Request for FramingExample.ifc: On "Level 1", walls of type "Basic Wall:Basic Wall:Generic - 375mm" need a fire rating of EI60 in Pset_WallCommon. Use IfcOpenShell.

First a look at what the model holds.

```python
import ifcopenshell
import ifcopenshell.util.element

model = ifcopenshell.open("FramingExample.ifc")
print(model.schema)
storey = next(s for s in model.by_type("IfcBuildingStorey") if s.Name == "Level 1")
walls = [e for e in ifcopenshell.util.element.get_decomposition(storey) if e.is_a("IfcWall")]
seen = {}
for e in walls:
    element_type = ifcopenshell.util.element.get_type(e)
    key = (element_type.Name if element_type != e and element_type else None, ifcopenshell.util.element.get_pset(e, "Pset_WallCommon", "FireRating"))
    seen[key] = seen.get(key, 0) + 1
for (name, value), count in sorted(seen.items(), key=str):
    print(count, "x", name, "|", value)
```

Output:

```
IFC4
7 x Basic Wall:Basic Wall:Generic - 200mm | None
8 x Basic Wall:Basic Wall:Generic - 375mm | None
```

```python
import ifcopenshell
import ifcopenshell.api.pset
import ifcopenshell.util.element

model = ifcopenshell.open("FramingExample.ifc")

storey = next(s for s in model.by_type("IfcBuildingStorey") if s.Name == "Level 1")
walls = [e for e in ifcopenshell.util.element.get_decomposition(storey) if e.is_a("IfcWall")]

count = 0
for e in walls:
    element_type = ifcopenshell.util.element.get_type(e)
    if element_type in (None, e) or element_type.Name != "Basic Wall:Basic Wall:Generic - 375mm":
        continue
    # add_pset returns the element's existing set when there is one.
    pset = ifcopenshell.api.pset.add_pset(model, product=e, name="Pset_WallCommon")
    ifcopenshell.api.pset.edit_pset(model, pset=pset, properties={"FireRating": "EI60"})
    count += 1

print(count, "walls updated")

model.write("FramingExample-out.ifc")
```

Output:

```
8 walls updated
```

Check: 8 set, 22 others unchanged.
